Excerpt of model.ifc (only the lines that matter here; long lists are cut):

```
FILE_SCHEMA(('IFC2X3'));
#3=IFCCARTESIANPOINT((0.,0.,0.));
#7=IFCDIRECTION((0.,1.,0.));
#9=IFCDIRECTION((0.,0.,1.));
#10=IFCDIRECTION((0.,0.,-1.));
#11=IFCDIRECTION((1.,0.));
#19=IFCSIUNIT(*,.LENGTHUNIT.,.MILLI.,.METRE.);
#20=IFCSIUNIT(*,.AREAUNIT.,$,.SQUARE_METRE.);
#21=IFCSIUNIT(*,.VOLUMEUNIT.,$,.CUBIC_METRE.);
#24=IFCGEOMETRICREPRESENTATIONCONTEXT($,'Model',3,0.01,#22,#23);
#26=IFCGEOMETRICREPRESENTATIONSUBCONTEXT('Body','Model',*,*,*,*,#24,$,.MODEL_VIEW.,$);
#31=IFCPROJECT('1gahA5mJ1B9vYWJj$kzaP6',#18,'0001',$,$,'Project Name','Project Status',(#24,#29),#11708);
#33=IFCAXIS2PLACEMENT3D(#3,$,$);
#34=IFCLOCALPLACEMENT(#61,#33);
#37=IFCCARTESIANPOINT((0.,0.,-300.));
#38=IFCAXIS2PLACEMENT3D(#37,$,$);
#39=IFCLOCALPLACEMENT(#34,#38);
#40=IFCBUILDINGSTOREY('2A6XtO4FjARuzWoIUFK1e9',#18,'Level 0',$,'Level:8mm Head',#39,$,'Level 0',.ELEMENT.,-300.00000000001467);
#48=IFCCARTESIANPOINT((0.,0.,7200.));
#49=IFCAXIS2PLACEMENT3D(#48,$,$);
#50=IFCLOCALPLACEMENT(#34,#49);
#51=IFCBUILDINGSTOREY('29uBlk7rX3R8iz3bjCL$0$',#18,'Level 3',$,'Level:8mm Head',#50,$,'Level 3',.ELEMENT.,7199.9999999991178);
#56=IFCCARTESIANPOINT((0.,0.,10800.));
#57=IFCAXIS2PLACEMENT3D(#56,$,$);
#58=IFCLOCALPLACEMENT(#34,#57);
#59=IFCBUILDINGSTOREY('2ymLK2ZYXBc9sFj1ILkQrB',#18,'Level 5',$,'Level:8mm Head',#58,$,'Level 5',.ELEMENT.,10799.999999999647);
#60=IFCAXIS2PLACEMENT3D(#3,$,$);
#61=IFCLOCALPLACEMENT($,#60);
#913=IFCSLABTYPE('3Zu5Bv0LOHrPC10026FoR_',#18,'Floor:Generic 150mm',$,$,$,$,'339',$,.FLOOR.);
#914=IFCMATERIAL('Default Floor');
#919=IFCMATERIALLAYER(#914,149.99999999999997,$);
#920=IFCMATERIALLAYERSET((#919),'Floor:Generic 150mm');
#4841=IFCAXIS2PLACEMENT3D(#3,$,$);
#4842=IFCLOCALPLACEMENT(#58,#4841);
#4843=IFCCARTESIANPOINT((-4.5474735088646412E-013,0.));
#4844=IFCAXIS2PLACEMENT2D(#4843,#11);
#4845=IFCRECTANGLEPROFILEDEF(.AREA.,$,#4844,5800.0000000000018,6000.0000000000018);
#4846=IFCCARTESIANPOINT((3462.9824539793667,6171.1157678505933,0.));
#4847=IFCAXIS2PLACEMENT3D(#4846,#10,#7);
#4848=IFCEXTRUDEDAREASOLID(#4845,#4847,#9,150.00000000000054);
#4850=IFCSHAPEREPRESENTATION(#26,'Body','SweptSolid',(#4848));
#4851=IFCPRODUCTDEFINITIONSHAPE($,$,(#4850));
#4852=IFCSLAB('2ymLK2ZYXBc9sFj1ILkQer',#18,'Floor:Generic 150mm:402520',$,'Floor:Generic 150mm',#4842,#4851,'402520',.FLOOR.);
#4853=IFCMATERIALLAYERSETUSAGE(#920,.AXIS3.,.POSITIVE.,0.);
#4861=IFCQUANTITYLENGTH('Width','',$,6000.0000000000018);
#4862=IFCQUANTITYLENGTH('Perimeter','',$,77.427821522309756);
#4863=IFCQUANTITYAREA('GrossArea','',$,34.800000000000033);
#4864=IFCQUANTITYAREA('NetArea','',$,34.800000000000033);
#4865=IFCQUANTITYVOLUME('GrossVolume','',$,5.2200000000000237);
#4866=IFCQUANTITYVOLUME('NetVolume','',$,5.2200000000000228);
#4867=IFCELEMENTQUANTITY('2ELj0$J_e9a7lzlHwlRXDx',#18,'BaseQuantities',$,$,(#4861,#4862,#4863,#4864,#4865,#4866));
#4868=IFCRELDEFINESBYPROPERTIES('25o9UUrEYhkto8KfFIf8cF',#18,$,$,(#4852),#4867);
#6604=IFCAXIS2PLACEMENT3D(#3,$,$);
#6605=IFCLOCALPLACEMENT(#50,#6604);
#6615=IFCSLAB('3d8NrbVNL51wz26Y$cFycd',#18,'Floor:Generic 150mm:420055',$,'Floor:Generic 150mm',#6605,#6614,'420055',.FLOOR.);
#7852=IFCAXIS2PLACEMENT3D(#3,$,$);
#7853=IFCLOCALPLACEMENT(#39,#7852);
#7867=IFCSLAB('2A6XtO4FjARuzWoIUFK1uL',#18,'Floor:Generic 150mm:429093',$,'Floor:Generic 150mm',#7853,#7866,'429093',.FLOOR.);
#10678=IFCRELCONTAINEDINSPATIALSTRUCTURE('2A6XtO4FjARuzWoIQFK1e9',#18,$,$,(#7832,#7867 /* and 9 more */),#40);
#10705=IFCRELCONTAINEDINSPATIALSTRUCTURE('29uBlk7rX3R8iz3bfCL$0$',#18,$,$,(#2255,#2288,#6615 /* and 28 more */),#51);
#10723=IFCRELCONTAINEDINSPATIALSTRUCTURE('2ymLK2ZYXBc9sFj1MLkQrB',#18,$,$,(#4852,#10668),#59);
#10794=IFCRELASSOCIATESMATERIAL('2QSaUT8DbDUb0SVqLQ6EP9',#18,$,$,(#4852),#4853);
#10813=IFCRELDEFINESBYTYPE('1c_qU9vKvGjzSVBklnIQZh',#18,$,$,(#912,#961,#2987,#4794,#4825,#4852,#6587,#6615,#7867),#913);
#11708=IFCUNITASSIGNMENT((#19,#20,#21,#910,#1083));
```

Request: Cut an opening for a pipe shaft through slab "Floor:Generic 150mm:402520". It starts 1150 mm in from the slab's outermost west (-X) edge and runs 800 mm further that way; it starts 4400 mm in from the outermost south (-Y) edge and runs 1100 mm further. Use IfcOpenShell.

```python
import numpy as np
import ifcopenshell
import ifcopenshell.api.feature
import ifcopenshell.api.geometry
import ifcopenshell.api.pset
import ifcopenshell.api.root
import ifcopenshell.geom
import ifcopenshell.util.element
import ifcopenshell.util.placement
import ifcopenshell.util.representation
import ifcopenshell.util.shape
import ifcopenshell.util.unit

model = ifcopenshell.open("model.ifc")
unit_scale = ifcopenshell.util.unit.calculate_unit_scale(model)
area_scale = ifcopenshell.util.unit.calculate_unit_scale(model, "AREAUNIT")
volume_scale = ifcopenshell.util.unit.calculate_unit_scale(model, "VOLUMEUNIT")
settings = ifcopenshell.geom.settings()


def volume(element):
    """Net volume in cubic metres, openings subtracted."""
    shape = ifcopenshell.geom.create_shape(settings, element)
    return ifcopenshell.util.shape.get_volume(shape.geometry)


slab = model.by_id(4852)
before = volume(slab)

# Extent in the slab's own axes, in metres. The edges named are its -X and -Y sides.
slab_shape = ifcopenshell.geom.create_shape(settings, slab)
vertices = ifcopenshell.util.shape.get_vertices(slab_shape.geometry)
x_min, y_min, bottom = vertices.min(axis=0)
top = vertices[:, 2].max()

opening = ifcopenshell.api.root.create_entity(model, ifc_class="IfcOpeningElement", name="Pipe shaft opening")
context = ifcopenshell.util.representation.get_context(model, "Model", "Body", "MODEL_VIEW")
width, depth = 0.8, 1.1
outline = [(0.0, 0.0), (width, 0.0), (width, depth), (0.0, depth), (0.0, 0.0)]
# Overshoot both faces by 50 mm so the cut is clean.
shape = ifcopenshell.api.geometry.add_slab_representation(
    model, context=context, depth=top - bottom + 0.1, polyline=outline
)
ifcopenshell.api.geometry.assign_representation(model, product=opening, representation=shape)

matrix = ifcopenshell.util.placement.get_local_placement(slab.ObjectPlacement)
matrix[:, 3] = matrix @ np.append(np.array([x_min + 1.15, y_min + 4.4, bottom - 0.05]) / unit_scale, 1.0)
ifcopenshell.api.geometry.edit_object_placement(model, product=opening, matrix=matrix, is_si=False)
ifcopenshell.api.feature.add_feature(model, feature=opening, element=slab)

after = volume(slab)

# Update the slab's stored quantities.
qto = model.by_id(ifcopenshell.util.element.get_pset(slab, "BaseQuantities", should_inherit=False)["id"])
ifcopenshell.api.pset.edit_qto(model, qto=qto, properties={
    "NetArea": after / (top - bottom) / area_scale,
    "NetVolume": after / volume_scale,
})

print(f"slab volume {before:.3f} -> {after:.3f} m3")

model.write("model_v2.ifc")
```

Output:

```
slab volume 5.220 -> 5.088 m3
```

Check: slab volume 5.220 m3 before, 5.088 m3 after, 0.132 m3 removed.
